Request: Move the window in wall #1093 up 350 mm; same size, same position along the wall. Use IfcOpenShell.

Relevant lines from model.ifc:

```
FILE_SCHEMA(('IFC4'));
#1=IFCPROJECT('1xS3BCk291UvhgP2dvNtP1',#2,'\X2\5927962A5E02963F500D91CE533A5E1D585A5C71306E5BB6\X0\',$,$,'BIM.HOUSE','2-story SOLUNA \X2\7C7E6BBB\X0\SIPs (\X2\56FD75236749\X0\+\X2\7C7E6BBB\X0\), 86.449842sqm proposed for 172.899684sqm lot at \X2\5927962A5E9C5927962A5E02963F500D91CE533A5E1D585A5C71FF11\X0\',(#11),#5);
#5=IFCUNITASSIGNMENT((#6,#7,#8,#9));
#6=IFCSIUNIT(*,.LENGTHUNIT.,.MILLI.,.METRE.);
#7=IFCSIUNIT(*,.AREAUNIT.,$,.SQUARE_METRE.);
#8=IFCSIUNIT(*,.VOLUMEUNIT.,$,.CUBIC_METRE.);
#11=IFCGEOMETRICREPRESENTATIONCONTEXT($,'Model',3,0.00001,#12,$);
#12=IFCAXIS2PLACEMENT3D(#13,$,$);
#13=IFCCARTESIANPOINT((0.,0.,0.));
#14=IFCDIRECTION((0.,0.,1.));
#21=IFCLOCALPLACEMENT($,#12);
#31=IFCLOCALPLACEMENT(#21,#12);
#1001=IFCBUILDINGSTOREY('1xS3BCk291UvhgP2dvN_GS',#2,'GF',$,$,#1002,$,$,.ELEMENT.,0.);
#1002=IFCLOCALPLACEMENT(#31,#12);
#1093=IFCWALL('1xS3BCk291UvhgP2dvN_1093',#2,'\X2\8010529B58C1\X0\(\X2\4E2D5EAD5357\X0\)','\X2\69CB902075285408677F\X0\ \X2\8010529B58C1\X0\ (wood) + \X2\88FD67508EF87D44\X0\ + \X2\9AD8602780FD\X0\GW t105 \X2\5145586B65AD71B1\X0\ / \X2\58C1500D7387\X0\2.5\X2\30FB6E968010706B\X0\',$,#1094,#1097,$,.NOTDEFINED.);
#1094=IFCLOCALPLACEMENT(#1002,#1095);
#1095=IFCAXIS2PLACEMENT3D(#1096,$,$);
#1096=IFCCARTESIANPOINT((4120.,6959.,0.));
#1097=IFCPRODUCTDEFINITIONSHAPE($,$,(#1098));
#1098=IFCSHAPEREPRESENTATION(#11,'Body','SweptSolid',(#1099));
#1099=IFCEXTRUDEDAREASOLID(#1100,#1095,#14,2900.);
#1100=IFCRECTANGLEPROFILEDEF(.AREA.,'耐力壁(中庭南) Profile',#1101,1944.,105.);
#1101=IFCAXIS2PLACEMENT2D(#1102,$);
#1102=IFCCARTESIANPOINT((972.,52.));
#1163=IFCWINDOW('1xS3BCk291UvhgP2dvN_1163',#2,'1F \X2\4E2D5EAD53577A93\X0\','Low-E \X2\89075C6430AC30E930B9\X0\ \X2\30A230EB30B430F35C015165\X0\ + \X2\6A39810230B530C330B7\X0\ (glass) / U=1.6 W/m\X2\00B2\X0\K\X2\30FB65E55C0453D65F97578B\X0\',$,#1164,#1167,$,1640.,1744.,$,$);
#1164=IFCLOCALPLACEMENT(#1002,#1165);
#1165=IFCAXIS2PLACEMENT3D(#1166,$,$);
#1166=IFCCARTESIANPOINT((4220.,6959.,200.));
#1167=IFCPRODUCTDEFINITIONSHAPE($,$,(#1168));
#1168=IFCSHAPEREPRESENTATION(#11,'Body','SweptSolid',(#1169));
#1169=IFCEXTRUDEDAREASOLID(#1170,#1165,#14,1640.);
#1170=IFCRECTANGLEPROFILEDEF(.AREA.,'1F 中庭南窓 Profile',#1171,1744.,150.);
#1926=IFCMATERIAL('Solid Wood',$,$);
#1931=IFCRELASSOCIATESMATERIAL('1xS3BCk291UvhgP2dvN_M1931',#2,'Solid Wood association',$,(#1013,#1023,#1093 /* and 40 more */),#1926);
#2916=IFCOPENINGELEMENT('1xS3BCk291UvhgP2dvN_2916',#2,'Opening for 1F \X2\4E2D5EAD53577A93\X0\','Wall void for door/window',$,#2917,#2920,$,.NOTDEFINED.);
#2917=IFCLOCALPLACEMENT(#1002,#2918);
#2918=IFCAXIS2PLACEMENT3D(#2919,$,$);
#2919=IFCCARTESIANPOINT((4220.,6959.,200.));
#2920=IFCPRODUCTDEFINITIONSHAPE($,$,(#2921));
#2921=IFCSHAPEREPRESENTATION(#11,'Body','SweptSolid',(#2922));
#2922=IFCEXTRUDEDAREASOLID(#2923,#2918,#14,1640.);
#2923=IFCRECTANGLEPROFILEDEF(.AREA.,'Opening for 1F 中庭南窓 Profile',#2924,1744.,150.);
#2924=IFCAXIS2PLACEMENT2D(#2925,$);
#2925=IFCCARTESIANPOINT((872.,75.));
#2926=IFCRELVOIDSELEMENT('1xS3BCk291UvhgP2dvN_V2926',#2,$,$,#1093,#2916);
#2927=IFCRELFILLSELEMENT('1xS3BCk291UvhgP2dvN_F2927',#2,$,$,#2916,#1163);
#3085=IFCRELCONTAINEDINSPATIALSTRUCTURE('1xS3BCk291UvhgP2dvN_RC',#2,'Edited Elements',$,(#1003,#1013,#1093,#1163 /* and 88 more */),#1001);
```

```python
import numpy as np
import ifcopenshell
import ifcopenshell.api.geometry
import ifcopenshell.util.placement
import ifcopenshell.util.unit

model = ifcopenshell.open("model.ifc")
unit_scale = ifcopenshell.util.unit.calculate_unit_scale(model)

window = model.by_id(1163)
opening = window.FillsVoids[0].RelatingOpeningElement
dz = 0.35 / unit_scale

shift = np.array([0.0, 0.0, dz])
# The window is not placed relative to its opening, so move both.
for product in (opening, window):
    matrix = ifcopenshell.util.placement.get_local_placement(product.ObjectPlacement)
    matrix[:3, 3] += shift
    ifcopenshell.api.geometry.edit_object_placement(model, product=product, matrix=matrix, is_si=False)

print(f"moved by {dz * unit_scale:+.3f} m")

model.write("model_v2.ifc")
```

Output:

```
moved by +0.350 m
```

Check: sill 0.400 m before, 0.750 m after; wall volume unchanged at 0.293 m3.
